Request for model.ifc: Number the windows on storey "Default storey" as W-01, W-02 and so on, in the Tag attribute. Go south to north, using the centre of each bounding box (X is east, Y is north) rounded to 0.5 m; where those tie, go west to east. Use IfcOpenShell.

First a look at what the model holds.

```python
import ifcopenshell
import ifcopenshell.util.element
import ifcopenshell.util.placement

model = ifcopenshell.open("model.ifc")
print(model.schema)
storey = next(s for s in model.by_type("IfcBuildingStorey") if s.Name == "Default storey")
windows = [e for e in ifcopenshell.util.element.get_decomposition(storey) if e.is_a("IfcWindow")]
for e in sorted(windows, key=lambda e: e.id()):
    origin = ifcopenshell.util.placement.get_local_placement(e.ObjectPlacement)[:3, 3]
    print(e.id(), e.Tag, e.Name, origin.round(2) + 0.0, sep=" | ")
```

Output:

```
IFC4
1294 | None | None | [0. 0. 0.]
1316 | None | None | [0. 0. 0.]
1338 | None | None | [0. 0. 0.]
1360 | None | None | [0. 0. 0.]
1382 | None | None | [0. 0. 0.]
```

```python
import ifcopenshell
import ifcopenshell.geom
import ifcopenshell.util.element
import ifcopenshell.util.shape

model = ifcopenshell.open("model.ifc")
settings = ifcopenshell.geom.settings()
settings.set("use-world-coords", True)


def centre(element):
    shape = ifcopenshell.geom.create_shape(settings, element)
    return ifcopenshell.util.shape.get_bbox_centroid(shape.geometry)


storey = next(s for s in model.by_type("IfcBuildingStorey") if s.Name == "Default storey")
windows = [e for e in ifcopenshell.util.element.get_decomposition(storey) if e.is_a("IfcWindow")]

# Insertion points can sit at a corner or the storey origin, so sort by the geometry (in metres).
centres = {e: centre(e) for e in windows}
windows.sort(key=lambda e: (round(centres[e][1] / 0.5), centres[e][0]))

for i, e in enumerate(windows, start=1):
    number = f"W-{i:02d}"
    e.Tag = number
    print(e.id(), number)

model.write("model_v2.ifc")
```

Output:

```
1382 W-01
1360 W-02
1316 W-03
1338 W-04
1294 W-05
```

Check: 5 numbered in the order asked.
